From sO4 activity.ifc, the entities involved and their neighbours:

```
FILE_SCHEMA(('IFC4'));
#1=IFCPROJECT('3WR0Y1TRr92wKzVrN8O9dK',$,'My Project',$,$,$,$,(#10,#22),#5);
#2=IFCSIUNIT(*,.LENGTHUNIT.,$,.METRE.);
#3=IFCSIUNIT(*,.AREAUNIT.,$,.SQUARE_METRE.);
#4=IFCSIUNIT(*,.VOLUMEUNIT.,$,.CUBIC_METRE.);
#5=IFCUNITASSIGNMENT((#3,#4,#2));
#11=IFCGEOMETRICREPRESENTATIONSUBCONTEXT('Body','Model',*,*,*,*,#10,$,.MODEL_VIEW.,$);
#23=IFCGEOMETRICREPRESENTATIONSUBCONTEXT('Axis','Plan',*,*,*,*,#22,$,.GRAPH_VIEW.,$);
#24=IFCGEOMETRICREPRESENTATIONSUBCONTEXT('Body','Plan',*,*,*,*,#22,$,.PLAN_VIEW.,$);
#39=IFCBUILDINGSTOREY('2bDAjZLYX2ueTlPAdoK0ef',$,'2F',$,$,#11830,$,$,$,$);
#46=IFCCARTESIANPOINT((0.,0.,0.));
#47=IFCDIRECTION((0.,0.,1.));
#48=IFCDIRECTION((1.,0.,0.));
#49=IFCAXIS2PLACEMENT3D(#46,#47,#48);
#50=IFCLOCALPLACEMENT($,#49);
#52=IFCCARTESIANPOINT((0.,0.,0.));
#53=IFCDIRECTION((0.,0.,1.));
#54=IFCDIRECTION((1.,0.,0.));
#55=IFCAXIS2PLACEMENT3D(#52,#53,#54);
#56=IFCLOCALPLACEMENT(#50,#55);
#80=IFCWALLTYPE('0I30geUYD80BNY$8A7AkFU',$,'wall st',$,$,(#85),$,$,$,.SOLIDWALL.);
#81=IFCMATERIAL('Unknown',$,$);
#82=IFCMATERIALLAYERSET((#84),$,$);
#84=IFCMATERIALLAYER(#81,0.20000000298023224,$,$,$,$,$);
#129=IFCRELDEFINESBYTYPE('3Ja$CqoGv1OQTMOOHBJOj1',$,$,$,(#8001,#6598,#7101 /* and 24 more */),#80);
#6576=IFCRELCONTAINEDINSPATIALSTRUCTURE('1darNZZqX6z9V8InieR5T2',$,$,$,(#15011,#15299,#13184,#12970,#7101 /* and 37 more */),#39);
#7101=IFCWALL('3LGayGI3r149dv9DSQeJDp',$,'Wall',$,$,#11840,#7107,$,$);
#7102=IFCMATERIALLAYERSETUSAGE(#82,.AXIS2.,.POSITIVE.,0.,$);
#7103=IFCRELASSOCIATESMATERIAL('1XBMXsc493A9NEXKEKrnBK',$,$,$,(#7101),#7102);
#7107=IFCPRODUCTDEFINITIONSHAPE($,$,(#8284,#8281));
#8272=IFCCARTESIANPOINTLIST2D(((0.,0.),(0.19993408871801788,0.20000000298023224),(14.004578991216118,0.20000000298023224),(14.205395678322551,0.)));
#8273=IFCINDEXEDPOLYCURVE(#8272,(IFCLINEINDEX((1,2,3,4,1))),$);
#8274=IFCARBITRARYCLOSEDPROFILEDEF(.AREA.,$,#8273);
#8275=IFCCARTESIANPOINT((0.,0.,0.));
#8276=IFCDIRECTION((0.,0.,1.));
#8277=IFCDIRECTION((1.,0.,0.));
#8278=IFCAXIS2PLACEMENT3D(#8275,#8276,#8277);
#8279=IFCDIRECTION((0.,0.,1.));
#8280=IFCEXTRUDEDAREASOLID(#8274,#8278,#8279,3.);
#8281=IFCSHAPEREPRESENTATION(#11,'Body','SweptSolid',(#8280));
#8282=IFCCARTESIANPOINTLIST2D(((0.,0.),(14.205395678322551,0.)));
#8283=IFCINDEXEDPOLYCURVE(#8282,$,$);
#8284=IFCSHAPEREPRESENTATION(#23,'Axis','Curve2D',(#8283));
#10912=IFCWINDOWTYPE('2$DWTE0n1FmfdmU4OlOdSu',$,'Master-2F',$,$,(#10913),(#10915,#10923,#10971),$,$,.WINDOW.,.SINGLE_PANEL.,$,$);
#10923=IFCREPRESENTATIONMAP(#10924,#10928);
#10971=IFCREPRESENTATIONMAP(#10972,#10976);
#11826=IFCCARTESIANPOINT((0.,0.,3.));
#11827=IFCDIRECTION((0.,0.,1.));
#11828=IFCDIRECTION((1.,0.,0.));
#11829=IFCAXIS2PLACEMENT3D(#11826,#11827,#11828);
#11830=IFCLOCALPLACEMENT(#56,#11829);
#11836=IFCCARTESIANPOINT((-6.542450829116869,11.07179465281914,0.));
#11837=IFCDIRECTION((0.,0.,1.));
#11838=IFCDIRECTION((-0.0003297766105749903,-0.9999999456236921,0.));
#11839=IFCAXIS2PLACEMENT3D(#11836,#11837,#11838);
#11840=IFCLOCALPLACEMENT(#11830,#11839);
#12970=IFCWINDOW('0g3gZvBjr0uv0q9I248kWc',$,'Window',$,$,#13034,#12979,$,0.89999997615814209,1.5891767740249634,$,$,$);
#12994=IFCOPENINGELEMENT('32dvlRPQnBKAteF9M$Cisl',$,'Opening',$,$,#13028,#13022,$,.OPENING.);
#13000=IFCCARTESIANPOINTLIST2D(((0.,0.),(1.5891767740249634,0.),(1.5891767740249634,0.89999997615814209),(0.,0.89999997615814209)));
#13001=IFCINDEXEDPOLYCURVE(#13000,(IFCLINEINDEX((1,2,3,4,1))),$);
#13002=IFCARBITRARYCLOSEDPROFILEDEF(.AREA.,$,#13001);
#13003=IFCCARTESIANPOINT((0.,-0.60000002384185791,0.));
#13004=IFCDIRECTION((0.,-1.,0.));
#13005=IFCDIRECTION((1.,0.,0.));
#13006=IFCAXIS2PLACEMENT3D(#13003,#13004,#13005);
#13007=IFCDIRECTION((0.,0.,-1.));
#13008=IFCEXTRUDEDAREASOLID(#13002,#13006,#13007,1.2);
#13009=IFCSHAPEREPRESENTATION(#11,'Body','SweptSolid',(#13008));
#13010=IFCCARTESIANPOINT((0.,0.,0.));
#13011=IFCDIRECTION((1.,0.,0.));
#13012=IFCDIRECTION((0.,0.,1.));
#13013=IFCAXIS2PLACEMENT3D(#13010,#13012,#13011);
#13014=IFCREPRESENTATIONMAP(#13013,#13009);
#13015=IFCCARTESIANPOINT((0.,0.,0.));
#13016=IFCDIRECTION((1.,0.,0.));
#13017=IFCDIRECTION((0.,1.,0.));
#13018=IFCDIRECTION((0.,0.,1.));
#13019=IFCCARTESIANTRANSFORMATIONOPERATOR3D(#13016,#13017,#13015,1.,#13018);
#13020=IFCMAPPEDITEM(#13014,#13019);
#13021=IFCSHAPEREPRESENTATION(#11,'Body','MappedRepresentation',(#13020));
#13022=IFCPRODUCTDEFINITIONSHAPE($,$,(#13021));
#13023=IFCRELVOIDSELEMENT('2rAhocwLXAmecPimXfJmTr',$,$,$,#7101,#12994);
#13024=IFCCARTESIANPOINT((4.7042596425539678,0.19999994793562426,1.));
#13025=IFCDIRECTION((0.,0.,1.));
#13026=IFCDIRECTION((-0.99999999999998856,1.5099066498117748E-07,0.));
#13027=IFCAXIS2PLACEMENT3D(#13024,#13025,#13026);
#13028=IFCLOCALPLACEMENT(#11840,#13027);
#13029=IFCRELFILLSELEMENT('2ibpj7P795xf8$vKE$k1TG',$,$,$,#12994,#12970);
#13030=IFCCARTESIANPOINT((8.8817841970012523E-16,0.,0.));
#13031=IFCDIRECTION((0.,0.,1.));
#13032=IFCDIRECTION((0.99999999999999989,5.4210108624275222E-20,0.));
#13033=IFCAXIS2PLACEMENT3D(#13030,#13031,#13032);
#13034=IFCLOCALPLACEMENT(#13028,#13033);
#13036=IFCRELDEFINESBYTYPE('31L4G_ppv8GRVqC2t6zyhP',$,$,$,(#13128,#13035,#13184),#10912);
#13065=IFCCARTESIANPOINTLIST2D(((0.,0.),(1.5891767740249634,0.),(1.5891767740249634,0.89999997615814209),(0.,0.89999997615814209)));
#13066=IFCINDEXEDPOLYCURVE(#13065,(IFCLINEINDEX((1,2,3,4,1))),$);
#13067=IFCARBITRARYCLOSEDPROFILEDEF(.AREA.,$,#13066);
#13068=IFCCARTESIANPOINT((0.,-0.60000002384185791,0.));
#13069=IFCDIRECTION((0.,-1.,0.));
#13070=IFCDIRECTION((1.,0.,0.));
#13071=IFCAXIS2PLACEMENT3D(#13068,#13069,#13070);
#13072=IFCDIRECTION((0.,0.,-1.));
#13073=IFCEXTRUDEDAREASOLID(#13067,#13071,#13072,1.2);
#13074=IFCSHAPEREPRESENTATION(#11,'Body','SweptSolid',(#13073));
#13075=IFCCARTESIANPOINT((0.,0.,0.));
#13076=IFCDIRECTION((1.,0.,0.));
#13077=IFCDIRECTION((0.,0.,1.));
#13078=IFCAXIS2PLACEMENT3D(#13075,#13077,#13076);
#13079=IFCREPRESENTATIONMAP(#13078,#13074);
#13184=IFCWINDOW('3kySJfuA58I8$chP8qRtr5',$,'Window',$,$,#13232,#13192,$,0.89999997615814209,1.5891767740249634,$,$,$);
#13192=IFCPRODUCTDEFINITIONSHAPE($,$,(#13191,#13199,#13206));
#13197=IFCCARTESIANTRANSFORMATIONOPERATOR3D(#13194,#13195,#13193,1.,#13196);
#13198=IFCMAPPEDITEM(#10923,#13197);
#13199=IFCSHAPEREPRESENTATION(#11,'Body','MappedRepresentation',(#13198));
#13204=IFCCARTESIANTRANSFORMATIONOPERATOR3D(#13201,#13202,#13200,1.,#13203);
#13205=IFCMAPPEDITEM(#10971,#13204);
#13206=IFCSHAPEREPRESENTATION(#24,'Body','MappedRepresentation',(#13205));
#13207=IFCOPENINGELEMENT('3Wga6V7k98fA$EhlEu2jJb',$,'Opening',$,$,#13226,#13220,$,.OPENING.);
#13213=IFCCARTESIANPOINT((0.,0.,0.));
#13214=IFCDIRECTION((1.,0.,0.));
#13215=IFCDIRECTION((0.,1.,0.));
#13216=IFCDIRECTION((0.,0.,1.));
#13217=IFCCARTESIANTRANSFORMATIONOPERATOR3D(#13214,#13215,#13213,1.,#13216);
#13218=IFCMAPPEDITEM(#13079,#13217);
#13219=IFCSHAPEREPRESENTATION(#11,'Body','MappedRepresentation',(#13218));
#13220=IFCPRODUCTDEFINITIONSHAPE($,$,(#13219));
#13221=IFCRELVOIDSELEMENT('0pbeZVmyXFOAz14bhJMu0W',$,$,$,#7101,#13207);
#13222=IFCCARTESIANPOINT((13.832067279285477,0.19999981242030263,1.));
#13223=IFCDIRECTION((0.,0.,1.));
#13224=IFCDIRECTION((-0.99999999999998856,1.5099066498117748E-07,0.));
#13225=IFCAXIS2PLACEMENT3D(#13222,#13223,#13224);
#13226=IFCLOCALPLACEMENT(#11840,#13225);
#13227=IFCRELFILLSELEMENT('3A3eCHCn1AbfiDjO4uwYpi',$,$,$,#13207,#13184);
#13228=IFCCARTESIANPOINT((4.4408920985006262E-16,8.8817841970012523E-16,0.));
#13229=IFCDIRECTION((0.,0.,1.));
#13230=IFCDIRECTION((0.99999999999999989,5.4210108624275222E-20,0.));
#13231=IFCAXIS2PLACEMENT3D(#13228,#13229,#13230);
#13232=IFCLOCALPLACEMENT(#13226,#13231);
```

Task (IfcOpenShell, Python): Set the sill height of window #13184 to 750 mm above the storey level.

```python
import numpy as np
import ifcopenshell
import ifcopenshell.api.geometry
import ifcopenshell.geom
import ifcopenshell.util.element
import ifcopenshell.util.placement
import ifcopenshell.util.shape
import ifcopenshell.util.unit

model = ifcopenshell.open("sO4 activity.ifc")
unit_scale = ifcopenshell.util.unit.calculate_unit_scale(model)

window = model.by_guid("3kySJfuA58I8$chP8qRtr5")
opening = window.FillsVoids[0].RelatingOpeningElement
storey = ifcopenshell.util.element.get_container(window, ifc_class="IfcBuildingStorey")
level = ifcopenshell.util.placement.get_local_placement(storey.ObjectPlacement)[2, 3]

# The opening's origin need not be at the sill, so measure its lowest point.
shape = ifcopenshell.geom.create_shape(ifcopenshell.geom.settings(), opening)
bottom = ifcopenshell.util.shape.get_shape_bottom_elevation(shape, shape.geometry) / unit_scale
dz = level + 0.75 - bottom

shift = np.array([0.0, 0.0, dz])
# The window is placed relative to its opening, so it follows when the opening moves.
matrix = ifcopenshell.util.placement.get_local_placement(opening.ObjectPlacement)
matrix[:3, 3] += shift
ifcopenshell.api.geometry.edit_object_placement(
    model, product=opening, matrix=matrix, is_si=False, should_transform_children=True
)

print(f"moved by {dz * unit_scale:+.3f} m")

model.write("sO4 activity-out.ifc")
```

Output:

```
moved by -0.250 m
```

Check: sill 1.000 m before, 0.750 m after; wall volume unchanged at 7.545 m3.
